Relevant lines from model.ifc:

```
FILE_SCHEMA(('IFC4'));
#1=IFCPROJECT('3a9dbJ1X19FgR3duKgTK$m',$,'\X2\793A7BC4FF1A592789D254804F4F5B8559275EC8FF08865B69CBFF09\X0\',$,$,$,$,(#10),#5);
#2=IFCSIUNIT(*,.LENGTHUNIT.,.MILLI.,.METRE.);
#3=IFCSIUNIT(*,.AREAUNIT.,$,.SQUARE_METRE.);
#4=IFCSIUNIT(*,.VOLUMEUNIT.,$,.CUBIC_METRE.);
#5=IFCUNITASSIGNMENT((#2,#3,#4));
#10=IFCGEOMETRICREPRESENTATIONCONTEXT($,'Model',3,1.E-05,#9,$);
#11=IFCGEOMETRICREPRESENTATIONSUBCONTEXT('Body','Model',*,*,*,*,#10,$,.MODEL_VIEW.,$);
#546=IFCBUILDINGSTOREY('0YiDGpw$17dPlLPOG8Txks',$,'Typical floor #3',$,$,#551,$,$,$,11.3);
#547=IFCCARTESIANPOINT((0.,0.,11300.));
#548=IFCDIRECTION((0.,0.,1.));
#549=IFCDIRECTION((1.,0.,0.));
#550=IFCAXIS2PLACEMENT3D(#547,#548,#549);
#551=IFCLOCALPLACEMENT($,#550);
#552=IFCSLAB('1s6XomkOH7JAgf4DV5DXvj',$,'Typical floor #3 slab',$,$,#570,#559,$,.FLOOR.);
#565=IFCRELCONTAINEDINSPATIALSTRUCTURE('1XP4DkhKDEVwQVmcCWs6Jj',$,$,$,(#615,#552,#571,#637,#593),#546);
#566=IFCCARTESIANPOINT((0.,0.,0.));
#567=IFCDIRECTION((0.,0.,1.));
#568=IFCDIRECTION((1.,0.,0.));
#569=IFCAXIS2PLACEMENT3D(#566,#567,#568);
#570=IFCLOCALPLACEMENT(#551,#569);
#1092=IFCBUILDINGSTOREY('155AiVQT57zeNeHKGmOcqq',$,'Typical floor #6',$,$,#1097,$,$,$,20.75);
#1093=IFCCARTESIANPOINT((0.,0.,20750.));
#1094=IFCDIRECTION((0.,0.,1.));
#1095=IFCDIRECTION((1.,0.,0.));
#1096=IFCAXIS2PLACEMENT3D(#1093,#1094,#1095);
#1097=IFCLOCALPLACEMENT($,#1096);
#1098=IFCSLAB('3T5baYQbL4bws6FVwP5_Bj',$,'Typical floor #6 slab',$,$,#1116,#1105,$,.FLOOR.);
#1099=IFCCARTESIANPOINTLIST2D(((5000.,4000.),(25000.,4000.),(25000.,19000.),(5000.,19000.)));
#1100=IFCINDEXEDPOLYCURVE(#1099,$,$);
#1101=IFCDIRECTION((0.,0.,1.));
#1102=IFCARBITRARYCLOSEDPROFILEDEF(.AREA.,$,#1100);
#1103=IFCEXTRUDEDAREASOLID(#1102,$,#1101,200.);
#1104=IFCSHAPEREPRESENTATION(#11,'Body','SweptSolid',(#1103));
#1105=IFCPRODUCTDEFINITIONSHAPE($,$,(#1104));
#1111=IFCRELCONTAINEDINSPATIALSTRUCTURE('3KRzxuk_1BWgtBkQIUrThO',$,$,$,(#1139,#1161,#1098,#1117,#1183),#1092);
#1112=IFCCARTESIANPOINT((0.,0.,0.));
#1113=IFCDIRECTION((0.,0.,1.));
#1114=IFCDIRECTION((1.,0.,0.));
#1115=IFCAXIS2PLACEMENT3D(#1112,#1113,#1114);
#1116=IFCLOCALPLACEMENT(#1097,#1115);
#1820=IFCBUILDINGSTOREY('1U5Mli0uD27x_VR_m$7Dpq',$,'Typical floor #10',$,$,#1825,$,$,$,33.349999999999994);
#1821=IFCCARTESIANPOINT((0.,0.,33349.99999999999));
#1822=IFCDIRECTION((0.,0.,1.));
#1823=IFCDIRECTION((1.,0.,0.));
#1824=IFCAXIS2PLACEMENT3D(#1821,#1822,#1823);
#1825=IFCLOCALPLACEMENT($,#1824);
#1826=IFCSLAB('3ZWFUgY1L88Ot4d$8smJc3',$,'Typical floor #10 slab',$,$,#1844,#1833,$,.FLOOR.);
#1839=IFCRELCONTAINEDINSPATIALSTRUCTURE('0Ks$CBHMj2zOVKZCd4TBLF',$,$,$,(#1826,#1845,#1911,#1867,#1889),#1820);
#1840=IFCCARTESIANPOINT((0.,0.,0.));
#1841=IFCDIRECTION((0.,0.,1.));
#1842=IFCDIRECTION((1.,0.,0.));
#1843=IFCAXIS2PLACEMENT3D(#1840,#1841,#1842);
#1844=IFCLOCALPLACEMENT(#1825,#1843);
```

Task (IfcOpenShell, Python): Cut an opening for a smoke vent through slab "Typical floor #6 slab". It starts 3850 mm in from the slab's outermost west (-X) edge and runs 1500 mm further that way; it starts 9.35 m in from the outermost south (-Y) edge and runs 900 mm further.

```python
import numpy as np
import ifcopenshell
import ifcopenshell.api.feature
import ifcopenshell.api.geometry
import ifcopenshell.api.root
import ifcopenshell.geom
import ifcopenshell.util.placement
import ifcopenshell.util.representation
import ifcopenshell.util.shape
import ifcopenshell.util.unit

model = ifcopenshell.open("model.ifc")
unit_scale = ifcopenshell.util.unit.calculate_unit_scale(model)
settings = ifcopenshell.geom.settings()


def volume(element):
    """Net volume in cubic metres, openings subtracted."""
    shape = ifcopenshell.geom.create_shape(settings, element)
    return ifcopenshell.util.shape.get_volume(shape.geometry)


slab = model.by_id(1098)
before = volume(slab)

# Extent in the slab's own axes, in metres. The edges named are its -X and -Y sides.
slab_shape = ifcopenshell.geom.create_shape(settings, slab)
vertices = ifcopenshell.util.shape.get_vertices(slab_shape.geometry)
x_min, y_min, bottom = vertices.min(axis=0)
top = vertices[:, 2].max()

opening = ifcopenshell.api.root.create_entity(model, ifc_class="IfcOpeningElement", name="Smoke vent opening", predefined_type="OPENING")
context = ifcopenshell.util.representation.get_context(model, "Model", "Body", "MODEL_VIEW")
width, depth = 1.5, 0.9
outline = [(0.0, 0.0), (width, 0.0), (width, depth), (0.0, depth), (0.0, 0.0)]
# Overshoot both faces by 50 mm so the cut is clean.
shape = ifcopenshell.api.geometry.add_slab_representation(
    model, context=context, depth=top - bottom + 0.1, polyline=outline
)
ifcopenshell.api.geometry.assign_representation(model, product=opening, representation=shape)

matrix = ifcopenshell.util.placement.get_local_placement(slab.ObjectPlacement)
matrix[:, 3] = matrix @ np.append(np.array([x_min + 3.85, y_min + 9.35, bottom - 0.05]) / unit_scale, 1.0)
ifcopenshell.api.geometry.edit_object_placement(model, product=opening, matrix=matrix, is_si=False)
ifcopenshell.api.feature.add_feature(model, feature=opening, element=slab)

after = volume(slab)

print(f"slab volume {before:.3f} -> {after:.3f} m3")

model.write("model_edited.ifc")
```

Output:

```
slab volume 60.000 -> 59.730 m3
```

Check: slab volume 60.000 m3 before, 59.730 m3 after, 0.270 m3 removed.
